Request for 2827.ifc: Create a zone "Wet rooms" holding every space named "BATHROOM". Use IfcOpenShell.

First a look at what the model holds.

```python
import ifcopenshell

model = ifcopenshell.open("2827.ifc")
print(model.schema)
seen = {}
for space in model.by_type("IfcSpace"):
    seen[space.LongName] = seen.get(space.LongName, 0) + 1
for name, count in sorted(seen.items(), key=str):
    print(count, "x", name)
print("zones:", [z.Name for z in model.by_type("IfcZone")][:20])
```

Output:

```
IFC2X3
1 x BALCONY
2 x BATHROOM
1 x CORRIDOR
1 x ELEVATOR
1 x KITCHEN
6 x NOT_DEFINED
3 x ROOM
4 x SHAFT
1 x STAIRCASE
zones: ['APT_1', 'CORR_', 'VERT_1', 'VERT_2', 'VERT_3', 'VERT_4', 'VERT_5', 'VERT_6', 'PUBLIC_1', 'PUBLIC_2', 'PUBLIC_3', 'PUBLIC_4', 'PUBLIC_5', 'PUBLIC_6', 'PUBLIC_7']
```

```python
import ifcopenshell
import ifcopenshell.api.group
import ifcopenshell.api.root

model = ifcopenshell.open("2827.ifc")

names = {"BATHROOM"}
spaces = [s for s in model.by_type("IfcSpace") if s.LongName in names]

zone = ifcopenshell.api.root.create_entity(model, ifc_class="IfcZone", name="Wet rooms")
ifcopenshell.api.group.assign_group(model, products=spaces, group=zone)
print(len(spaces), "spaces in", zone.Name)

model.write("2827_v2.ifc")
```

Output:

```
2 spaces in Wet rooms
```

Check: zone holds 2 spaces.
